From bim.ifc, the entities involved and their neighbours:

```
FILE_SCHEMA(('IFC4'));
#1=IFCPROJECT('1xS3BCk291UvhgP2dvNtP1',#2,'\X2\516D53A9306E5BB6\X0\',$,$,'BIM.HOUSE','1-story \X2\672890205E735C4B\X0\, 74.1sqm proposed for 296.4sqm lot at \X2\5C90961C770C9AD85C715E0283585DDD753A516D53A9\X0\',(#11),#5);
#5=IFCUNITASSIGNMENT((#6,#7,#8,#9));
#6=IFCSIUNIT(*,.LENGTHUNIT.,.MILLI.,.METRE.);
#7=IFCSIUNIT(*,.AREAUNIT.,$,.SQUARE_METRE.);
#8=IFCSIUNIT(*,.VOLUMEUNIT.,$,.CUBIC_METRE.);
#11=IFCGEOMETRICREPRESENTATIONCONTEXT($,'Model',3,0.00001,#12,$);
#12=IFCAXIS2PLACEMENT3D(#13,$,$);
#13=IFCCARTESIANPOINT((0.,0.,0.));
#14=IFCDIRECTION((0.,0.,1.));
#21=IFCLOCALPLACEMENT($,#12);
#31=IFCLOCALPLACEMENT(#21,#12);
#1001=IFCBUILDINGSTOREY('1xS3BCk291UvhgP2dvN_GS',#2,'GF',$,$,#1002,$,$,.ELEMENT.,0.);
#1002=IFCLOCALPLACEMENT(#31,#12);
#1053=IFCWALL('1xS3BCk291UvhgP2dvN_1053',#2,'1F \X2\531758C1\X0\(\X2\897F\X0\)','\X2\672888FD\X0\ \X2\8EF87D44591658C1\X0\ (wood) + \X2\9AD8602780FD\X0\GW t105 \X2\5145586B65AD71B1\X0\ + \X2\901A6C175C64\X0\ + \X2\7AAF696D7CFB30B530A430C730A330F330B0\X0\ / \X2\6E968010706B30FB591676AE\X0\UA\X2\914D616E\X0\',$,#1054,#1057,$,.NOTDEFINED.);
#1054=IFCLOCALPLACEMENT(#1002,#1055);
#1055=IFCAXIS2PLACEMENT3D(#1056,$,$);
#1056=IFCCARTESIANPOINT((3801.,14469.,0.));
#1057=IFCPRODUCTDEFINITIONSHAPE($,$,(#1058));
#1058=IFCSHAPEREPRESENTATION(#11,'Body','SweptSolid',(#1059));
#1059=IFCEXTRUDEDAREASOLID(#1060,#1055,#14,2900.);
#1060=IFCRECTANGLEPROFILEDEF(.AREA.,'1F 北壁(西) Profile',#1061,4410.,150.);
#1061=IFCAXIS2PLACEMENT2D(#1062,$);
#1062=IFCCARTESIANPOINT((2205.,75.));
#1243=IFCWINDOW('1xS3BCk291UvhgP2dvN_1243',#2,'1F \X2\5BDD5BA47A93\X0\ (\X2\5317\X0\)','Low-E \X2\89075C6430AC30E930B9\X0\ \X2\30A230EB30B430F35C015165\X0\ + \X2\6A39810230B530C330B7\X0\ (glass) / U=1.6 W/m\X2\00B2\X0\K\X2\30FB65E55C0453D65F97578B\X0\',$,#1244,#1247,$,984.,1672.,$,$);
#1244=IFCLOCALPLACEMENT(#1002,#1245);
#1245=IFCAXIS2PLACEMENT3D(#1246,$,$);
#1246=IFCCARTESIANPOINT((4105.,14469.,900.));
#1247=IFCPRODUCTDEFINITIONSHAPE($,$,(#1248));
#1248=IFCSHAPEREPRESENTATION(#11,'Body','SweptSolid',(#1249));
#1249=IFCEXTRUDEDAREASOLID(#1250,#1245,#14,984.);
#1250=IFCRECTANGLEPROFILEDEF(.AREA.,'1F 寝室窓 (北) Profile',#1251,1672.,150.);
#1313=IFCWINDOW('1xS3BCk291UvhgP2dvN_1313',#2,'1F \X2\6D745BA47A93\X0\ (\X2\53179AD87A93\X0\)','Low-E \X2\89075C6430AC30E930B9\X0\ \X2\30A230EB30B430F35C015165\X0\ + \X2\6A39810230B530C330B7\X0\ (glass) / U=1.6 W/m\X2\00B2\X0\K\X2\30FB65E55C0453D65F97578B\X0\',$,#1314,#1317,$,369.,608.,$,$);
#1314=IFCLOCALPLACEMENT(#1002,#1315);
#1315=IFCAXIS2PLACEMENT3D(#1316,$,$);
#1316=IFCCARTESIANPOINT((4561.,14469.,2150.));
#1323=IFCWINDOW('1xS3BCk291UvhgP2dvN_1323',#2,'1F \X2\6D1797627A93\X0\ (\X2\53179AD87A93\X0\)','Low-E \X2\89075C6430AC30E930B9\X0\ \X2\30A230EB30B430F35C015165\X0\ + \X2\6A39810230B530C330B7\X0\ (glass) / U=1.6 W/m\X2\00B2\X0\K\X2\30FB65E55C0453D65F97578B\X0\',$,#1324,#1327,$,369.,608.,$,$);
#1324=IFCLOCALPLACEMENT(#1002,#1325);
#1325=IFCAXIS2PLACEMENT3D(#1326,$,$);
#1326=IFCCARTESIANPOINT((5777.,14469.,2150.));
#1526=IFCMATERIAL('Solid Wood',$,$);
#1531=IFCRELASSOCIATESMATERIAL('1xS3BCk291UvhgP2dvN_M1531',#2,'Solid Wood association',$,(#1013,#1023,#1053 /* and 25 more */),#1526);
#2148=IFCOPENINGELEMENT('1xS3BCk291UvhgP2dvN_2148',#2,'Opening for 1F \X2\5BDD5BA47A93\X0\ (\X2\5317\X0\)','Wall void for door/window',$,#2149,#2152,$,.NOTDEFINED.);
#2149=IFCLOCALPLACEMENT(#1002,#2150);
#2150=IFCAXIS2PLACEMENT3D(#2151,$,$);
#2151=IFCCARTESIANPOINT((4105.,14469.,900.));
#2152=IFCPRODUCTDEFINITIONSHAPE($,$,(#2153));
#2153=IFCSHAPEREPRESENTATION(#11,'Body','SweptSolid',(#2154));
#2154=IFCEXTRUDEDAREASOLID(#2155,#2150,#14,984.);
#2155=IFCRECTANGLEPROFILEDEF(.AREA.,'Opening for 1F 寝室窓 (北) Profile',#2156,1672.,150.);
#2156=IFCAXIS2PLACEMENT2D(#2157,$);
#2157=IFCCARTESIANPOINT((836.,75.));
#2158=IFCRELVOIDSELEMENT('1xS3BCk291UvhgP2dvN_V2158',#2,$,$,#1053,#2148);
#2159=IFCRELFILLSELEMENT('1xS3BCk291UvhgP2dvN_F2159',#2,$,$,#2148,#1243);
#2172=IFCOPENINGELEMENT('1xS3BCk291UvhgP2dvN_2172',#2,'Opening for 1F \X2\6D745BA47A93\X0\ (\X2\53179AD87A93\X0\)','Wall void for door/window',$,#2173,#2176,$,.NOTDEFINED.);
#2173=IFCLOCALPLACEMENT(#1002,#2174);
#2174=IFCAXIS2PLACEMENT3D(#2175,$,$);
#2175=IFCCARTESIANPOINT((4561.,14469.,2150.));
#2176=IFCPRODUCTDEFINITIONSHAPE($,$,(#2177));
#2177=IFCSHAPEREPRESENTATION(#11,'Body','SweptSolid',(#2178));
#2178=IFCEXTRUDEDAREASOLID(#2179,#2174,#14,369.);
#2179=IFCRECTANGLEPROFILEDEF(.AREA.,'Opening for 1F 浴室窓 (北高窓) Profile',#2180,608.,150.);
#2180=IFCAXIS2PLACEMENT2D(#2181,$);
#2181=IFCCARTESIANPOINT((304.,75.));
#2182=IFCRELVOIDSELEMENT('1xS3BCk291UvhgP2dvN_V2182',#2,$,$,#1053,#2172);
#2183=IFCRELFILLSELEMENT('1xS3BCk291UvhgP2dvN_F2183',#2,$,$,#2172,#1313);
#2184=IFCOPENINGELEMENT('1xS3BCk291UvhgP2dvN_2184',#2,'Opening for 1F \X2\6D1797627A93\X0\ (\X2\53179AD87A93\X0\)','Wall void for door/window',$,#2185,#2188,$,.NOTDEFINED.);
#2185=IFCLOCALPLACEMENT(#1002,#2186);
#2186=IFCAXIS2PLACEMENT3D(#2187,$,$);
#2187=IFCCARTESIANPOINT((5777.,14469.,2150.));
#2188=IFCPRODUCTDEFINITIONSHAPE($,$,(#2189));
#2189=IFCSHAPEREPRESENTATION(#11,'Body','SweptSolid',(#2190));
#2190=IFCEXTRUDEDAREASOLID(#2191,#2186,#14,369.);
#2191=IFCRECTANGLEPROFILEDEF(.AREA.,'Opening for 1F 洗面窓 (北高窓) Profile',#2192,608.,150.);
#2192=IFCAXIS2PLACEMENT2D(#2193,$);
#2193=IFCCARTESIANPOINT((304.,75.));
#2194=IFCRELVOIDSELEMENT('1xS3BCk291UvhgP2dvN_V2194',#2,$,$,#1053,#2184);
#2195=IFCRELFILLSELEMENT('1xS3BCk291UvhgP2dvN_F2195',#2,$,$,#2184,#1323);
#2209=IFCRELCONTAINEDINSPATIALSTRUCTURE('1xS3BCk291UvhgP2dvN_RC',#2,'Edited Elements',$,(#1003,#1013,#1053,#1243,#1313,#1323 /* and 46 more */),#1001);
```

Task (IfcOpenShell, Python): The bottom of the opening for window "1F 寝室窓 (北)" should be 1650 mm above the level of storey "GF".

```python
import numpy as np
import ifcopenshell
import ifcopenshell.api.geometry
import ifcopenshell.geom
import ifcopenshell.util.element
import ifcopenshell.util.placement
import ifcopenshell.util.shape
import ifcopenshell.util.unit

model = ifcopenshell.open("bim.ifc")
unit_scale = ifcopenshell.util.unit.calculate_unit_scale(model)

window = model.by_guid("1xS3BCk291UvhgP2dvN_1243")
opening = window.FillsVoids[0].RelatingOpeningElement
storey = ifcopenshell.util.element.get_container(window, ifc_class="IfcBuildingStorey")
level = ifcopenshell.util.placement.get_local_placement(storey.ObjectPlacement)[2, 3]

# The opening's origin need not be at the sill, so measure its lowest point.
shape = ifcopenshell.geom.create_shape(ifcopenshell.geom.settings(), opening)
bottom = ifcopenshell.util.shape.get_shape_bottom_elevation(shape, shape.geometry) / unit_scale
dz = level + 1.65 / unit_scale - bottom

shift = np.array([0.0, 0.0, dz])
# The window is not placed relative to its opening, so move both.
for product in (opening, window):
    matrix = ifcopenshell.util.placement.get_local_placement(product.ObjectPlacement)
    matrix[:3, 3] += shift
    ifcopenshell.api.geometry.edit_object_placement(model, product=product, matrix=matrix, is_si=False)

print(f"moved by {dz * unit_scale:+.3f} m")

model.write("bim-out.ifc")
```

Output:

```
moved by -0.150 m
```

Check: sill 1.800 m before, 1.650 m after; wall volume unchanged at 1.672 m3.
